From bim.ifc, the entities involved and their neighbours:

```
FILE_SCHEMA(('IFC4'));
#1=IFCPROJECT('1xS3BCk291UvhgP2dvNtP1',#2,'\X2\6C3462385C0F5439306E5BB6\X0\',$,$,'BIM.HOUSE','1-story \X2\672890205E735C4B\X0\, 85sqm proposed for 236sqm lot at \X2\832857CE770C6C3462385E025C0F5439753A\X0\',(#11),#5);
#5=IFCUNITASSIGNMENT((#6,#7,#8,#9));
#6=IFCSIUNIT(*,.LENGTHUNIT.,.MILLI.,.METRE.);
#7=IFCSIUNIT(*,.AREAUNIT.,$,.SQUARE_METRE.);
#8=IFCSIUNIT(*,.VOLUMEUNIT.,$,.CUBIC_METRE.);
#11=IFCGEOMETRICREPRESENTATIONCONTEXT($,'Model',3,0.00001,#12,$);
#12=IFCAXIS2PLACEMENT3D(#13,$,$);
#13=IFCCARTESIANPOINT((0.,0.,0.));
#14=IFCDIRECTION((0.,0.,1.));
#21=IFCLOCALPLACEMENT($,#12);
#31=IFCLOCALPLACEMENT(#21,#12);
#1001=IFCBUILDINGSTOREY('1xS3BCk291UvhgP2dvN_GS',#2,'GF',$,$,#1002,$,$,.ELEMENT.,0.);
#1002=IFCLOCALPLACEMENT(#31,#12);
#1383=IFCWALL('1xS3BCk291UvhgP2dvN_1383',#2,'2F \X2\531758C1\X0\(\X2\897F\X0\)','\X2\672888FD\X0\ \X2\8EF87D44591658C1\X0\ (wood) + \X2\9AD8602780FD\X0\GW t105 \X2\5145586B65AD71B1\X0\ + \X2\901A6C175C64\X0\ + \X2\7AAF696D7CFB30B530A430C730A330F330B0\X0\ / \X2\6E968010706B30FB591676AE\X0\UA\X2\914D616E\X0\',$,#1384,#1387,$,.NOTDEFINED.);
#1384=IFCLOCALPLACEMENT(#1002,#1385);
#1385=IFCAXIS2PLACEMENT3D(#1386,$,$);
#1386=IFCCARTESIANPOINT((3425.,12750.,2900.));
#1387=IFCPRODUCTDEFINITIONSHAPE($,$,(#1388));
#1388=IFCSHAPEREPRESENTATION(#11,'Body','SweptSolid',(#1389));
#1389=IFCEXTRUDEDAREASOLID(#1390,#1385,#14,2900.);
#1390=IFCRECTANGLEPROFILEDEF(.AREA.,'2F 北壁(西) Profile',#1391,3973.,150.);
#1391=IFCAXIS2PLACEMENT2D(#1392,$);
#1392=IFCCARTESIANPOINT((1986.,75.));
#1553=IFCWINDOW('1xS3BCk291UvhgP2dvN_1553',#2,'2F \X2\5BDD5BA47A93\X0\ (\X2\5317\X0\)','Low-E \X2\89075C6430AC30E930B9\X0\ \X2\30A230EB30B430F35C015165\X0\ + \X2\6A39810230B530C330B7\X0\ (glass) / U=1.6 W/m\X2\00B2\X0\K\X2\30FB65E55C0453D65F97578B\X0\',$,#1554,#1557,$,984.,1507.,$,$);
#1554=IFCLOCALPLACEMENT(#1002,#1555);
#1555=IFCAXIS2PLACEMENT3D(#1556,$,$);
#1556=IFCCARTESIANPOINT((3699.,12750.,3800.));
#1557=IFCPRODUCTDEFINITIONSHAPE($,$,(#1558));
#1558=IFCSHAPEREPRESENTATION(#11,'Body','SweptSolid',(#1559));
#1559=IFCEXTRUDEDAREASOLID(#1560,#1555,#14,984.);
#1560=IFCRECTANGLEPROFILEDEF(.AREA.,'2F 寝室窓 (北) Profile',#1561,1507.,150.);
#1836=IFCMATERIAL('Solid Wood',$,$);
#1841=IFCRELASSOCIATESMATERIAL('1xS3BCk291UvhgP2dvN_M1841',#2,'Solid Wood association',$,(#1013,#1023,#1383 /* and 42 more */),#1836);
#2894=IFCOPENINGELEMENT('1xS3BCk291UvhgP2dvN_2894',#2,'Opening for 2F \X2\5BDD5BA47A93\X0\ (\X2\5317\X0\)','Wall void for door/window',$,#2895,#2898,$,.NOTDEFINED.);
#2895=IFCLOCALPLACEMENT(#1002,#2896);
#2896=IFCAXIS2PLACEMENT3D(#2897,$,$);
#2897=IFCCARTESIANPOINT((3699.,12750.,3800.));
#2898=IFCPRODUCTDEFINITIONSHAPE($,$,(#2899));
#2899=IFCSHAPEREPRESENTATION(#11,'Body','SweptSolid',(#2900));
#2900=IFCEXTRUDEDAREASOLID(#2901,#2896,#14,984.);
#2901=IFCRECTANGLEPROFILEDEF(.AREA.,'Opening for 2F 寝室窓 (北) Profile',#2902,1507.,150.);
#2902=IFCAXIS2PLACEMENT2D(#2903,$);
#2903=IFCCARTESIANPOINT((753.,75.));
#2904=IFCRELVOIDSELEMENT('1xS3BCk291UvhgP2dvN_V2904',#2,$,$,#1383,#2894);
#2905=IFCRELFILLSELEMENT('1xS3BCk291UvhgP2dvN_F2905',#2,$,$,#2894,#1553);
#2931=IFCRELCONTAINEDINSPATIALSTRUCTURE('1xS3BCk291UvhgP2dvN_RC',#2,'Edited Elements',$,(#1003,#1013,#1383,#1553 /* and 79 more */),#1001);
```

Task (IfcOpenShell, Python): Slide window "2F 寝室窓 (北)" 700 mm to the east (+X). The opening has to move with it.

```python
import ifcopenshell
import ifcopenshell.api.geometry
import ifcopenshell.util.placement
import ifcopenshell.util.unit

model = ifcopenshell.open("bim.ifc")
unit_scale = ifcopenshell.util.unit.calculate_unit_scale(model)

window = model.by_guid("1xS3BCk291UvhgP2dvN_1553")
opening = window.FillsVoids[0].RelatingOpeningElement
wall = opening.VoidsElements[0].RelatingBuildingElement

wall_matrix = ifcopenshell.util.placement.get_local_placement(wall.ObjectPlacement)
shift = wall_matrix[:3, 0] * 0.7 / unit_scale
before = ifcopenshell.util.placement.get_local_placement(window.ObjectPlacement)[:3, 3].copy()

# The window is not placed relative to its opening, so move both.
for product in (opening, window):
    matrix = ifcopenshell.util.placement.get_local_placement(product.ObjectPlacement)
    matrix[:3, 3] += shift
    ifcopenshell.api.geometry.edit_object_placement(model, product=product, matrix=matrix, is_si=False)

after = ifcopenshell.util.placement.get_local_placement(window.ObjectPlacement)[:3, 3]
print("window moved by", (after - before).round(3) + 0.0)

model.write("bim_updated.ifc")
```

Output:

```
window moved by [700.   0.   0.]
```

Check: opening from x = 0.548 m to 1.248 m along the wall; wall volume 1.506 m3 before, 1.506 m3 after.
